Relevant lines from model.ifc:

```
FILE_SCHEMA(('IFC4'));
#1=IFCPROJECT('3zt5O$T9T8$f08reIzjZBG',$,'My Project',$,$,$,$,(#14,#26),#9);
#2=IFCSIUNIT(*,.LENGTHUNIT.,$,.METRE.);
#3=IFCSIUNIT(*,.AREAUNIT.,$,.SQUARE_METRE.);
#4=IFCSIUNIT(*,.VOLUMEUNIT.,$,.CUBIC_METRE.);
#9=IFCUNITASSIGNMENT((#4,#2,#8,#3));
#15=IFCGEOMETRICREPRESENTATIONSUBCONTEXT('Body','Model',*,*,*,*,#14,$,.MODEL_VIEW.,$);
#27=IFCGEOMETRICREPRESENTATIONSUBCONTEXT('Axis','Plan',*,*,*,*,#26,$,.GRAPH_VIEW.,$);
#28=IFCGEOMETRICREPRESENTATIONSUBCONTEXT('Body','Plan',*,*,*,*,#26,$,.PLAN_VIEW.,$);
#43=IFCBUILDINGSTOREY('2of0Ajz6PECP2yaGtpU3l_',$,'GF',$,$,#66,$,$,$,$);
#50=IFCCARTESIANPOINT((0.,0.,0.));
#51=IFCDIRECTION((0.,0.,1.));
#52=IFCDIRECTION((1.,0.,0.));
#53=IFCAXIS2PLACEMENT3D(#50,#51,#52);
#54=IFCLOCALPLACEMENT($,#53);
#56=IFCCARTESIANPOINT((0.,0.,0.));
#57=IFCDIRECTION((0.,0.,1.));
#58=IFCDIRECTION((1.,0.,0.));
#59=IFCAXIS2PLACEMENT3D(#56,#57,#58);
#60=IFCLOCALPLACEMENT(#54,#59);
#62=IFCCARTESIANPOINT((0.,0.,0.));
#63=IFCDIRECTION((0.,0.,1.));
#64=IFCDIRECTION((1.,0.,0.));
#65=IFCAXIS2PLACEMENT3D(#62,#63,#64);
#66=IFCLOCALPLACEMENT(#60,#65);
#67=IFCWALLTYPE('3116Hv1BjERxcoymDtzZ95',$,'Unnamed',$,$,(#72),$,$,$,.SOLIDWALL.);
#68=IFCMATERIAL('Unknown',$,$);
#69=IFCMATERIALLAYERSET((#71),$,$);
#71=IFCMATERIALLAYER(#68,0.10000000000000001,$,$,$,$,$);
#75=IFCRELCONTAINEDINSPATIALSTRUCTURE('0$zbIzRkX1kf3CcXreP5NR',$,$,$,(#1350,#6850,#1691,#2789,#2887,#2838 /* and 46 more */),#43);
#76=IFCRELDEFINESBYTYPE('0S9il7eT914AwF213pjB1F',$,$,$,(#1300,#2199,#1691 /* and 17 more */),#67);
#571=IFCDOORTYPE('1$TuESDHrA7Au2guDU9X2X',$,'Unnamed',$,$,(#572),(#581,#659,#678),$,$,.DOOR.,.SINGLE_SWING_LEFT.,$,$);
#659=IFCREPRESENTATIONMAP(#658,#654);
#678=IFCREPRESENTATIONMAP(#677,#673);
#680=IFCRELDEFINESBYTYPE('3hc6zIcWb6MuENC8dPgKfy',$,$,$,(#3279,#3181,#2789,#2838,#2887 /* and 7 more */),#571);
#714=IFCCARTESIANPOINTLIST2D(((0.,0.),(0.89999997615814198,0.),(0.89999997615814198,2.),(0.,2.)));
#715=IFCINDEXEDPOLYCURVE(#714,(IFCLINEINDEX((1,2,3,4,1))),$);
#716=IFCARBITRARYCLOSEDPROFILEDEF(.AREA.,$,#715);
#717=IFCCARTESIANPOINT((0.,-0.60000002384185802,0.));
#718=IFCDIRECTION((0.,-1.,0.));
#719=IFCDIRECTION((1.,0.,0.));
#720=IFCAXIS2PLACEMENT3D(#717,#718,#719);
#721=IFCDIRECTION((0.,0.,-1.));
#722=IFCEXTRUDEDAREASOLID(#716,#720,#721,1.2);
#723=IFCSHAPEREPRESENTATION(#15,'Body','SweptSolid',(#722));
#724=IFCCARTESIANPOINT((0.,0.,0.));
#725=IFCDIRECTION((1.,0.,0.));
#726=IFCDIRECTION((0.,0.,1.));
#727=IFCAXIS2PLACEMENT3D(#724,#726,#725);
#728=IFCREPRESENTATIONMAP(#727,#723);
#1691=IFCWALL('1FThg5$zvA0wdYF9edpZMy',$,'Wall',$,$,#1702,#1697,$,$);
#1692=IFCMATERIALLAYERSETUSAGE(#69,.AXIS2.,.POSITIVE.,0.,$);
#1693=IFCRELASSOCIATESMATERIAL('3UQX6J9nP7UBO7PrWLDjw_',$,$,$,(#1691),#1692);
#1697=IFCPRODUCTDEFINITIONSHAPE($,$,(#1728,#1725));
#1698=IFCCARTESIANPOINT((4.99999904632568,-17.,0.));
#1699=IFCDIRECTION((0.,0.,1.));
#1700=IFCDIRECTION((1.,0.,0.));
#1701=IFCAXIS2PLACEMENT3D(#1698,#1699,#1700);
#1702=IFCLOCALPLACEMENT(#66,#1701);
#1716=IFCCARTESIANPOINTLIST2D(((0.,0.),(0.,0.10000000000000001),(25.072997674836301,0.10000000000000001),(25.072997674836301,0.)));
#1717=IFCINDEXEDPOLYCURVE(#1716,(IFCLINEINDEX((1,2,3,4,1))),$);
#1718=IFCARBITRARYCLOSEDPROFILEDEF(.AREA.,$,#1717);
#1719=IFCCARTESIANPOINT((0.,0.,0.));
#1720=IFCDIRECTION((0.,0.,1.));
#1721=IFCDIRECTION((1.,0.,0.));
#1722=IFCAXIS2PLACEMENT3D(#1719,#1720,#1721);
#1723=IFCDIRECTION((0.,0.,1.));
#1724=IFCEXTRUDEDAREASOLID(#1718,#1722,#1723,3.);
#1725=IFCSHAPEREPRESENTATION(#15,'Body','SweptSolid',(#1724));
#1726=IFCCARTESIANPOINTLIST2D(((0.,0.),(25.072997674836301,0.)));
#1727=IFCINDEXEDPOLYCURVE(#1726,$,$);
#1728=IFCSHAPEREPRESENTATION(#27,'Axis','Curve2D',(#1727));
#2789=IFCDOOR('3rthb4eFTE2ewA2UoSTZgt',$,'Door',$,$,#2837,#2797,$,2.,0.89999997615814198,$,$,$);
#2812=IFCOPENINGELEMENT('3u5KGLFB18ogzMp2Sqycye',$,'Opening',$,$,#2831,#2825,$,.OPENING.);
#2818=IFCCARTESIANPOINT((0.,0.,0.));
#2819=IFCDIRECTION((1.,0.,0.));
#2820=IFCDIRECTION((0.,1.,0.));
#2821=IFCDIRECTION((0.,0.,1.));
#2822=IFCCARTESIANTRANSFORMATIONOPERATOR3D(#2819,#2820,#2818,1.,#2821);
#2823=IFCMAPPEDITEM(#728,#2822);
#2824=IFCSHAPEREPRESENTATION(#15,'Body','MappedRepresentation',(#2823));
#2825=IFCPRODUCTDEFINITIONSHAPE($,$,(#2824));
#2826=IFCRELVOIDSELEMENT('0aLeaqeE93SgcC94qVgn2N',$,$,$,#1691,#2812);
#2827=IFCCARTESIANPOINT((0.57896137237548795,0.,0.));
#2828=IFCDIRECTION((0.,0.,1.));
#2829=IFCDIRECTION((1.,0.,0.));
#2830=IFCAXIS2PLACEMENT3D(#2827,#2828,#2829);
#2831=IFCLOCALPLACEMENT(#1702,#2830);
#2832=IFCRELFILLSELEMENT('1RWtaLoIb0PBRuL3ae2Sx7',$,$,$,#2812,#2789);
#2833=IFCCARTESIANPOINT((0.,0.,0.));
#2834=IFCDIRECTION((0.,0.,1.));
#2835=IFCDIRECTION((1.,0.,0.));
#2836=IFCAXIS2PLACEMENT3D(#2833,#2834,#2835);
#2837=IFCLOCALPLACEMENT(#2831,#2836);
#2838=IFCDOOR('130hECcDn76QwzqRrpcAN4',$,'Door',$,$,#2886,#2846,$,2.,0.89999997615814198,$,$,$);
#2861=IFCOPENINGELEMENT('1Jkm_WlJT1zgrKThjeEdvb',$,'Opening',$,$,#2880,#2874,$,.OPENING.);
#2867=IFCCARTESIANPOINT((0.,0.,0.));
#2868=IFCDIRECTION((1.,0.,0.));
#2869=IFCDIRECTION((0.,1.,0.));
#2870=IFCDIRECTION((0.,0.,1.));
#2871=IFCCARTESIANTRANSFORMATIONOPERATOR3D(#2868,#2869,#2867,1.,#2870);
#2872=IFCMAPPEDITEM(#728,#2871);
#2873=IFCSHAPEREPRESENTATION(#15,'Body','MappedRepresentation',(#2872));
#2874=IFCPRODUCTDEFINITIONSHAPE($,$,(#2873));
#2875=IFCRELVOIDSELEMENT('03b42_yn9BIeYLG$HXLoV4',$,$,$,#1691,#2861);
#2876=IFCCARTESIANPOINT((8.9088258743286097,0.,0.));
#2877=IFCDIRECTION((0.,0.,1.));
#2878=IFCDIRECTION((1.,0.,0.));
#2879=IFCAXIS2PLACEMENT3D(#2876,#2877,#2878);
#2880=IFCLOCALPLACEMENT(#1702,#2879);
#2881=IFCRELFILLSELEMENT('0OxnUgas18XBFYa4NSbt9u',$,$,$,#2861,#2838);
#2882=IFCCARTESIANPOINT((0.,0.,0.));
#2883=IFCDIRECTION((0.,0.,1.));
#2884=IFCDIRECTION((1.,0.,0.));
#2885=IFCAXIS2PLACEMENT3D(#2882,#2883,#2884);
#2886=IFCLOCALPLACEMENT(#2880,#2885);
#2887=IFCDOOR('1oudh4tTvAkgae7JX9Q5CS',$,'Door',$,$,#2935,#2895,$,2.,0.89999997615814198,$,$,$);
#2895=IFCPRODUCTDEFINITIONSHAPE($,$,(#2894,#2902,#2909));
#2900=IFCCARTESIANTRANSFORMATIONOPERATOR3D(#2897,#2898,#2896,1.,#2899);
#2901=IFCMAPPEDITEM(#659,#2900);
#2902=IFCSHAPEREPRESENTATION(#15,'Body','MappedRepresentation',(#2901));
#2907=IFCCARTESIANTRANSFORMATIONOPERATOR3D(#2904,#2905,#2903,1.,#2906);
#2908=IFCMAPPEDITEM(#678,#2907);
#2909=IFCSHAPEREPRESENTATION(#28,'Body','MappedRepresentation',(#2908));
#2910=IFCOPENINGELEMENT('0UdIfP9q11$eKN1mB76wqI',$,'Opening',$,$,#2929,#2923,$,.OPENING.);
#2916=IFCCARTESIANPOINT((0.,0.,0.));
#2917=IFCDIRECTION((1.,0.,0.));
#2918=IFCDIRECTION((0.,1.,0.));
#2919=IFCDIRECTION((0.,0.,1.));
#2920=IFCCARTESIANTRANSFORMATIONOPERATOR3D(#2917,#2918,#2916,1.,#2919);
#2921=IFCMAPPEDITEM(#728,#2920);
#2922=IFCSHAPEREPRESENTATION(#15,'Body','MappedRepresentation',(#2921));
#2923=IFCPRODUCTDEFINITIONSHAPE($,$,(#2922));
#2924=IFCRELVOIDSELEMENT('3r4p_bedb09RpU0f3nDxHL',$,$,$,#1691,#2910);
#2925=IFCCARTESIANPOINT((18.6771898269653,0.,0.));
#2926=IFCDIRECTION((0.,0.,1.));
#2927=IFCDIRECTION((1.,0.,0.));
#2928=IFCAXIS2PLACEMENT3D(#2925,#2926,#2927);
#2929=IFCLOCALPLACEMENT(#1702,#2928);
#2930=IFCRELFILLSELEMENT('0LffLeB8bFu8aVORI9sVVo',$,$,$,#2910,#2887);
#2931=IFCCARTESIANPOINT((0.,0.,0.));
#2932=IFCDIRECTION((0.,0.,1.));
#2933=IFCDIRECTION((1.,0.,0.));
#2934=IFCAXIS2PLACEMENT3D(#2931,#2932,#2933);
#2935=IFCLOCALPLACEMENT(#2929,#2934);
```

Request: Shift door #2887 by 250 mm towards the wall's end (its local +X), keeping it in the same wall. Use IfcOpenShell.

```python
import ifcopenshell
import ifcopenshell.api.geometry
import ifcopenshell.util.placement
import ifcopenshell.util.unit

model = ifcopenshell.open("model.ifc")
unit_scale = ifcopenshell.util.unit.calculate_unit_scale(model)

door = model.by_id(2887)
opening = door.FillsVoids[0].RelatingOpeningElement
wall = opening.VoidsElements[0].RelatingBuildingElement

wall_matrix = ifcopenshell.util.placement.get_local_placement(wall.ObjectPlacement)
shift = wall_matrix[:3, 0] * 0.25 / unit_scale
before = ifcopenshell.util.placement.get_local_placement(door.ObjectPlacement)[:3, 3].copy()

# The door is placed relative to its opening, so it follows when the opening moves.
matrix = ifcopenshell.util.placement.get_local_placement(opening.ObjectPlacement)
matrix[:3, 3] += shift
ifcopenshell.api.geometry.edit_object_placement(
    model, product=opening, matrix=matrix, is_si=False, should_transform_children=True
)

after = ifcopenshell.util.placement.get_local_placement(door.ObjectPlacement)[:3, 3]
print("door moved by", (after - before).round(3) + 0.0)

model.write("model_edited.ifc")
```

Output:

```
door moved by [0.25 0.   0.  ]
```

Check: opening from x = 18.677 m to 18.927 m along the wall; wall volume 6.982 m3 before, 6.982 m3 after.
